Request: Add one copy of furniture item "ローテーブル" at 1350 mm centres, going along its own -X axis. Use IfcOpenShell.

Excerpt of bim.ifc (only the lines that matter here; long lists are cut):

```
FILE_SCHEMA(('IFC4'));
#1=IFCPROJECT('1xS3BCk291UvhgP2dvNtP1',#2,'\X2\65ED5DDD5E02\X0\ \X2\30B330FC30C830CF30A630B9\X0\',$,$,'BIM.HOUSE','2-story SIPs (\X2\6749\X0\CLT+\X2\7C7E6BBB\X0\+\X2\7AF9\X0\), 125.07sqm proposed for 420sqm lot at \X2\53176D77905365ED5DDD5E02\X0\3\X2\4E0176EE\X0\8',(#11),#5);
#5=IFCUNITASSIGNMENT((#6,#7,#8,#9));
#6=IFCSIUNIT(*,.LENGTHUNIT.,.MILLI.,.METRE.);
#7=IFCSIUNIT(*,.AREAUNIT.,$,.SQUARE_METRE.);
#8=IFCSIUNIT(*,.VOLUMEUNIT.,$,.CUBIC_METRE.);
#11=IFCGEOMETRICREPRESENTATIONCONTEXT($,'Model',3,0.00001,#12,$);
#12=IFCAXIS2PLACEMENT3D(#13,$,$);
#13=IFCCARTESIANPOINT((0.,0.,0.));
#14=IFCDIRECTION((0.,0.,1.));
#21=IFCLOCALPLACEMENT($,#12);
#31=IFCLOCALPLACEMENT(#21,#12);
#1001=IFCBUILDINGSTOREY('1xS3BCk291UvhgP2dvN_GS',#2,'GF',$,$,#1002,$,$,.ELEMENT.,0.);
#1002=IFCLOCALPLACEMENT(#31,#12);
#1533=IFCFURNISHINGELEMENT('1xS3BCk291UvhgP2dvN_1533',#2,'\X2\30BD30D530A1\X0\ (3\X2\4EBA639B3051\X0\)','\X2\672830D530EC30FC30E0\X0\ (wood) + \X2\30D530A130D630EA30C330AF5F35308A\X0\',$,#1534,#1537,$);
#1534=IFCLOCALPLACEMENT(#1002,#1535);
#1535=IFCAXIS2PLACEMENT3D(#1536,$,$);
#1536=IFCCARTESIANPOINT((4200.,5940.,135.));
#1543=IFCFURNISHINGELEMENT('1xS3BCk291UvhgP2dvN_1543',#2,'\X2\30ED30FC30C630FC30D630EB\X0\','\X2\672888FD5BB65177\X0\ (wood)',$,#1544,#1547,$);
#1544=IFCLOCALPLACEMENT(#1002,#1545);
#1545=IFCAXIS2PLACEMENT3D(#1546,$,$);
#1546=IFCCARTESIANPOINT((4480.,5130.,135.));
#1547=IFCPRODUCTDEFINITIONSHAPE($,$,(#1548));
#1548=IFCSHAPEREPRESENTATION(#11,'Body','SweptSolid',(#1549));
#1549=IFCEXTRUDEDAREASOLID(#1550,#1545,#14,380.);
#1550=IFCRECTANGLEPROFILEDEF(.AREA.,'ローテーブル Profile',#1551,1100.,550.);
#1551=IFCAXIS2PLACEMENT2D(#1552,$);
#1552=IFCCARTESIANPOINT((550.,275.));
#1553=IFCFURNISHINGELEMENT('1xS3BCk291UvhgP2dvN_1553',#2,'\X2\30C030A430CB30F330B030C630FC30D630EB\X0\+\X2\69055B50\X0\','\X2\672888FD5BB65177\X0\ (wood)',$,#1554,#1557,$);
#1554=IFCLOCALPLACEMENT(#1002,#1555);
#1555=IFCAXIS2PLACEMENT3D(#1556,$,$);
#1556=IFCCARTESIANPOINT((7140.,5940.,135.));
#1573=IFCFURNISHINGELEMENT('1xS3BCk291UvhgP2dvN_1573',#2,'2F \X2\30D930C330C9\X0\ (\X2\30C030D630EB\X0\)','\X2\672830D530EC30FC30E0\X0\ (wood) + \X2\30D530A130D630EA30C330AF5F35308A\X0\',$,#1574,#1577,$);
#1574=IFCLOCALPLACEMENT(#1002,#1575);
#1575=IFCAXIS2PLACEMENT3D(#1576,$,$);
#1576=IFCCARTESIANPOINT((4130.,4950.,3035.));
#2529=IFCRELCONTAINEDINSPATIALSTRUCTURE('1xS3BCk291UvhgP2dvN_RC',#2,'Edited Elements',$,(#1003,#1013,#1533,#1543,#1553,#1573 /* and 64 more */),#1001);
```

```python
import ifcopenshell
import ifcopenshell.api.geometry
import ifcopenshell.api.root
import ifcopenshell.util.element
import ifcopenshell.util.placement

model = ifcopenshell.open("bim.ifc")


def reuse_history(source, copy):
    """copy_class also copies each property set's owner history, people and application; keep the originals."""
    for rel in copy.IsDefinedBy:
        if rel.is_a("IfcRelDefinesByProperties") and (history := rel.RelatingPropertyDefinition.OwnerHistory):
            rel.RelatingPropertyDefinition.OwnerHistory = source.OwnerHistory
            ifcopenshell.util.element.remove_deep2(model, history)


source = model.by_guid("1xS3BCk291UvhgP2dvN_1543")
base = ifcopenshell.util.placement.get_local_placement(source.ObjectPlacement)
step = -base[:3, 0] * 1350.0

for i in range(1, 2):
    copy = ifcopenshell.api.root.copy_class(model, product=source)
    copy.Representation = ifcopenshell.util.element.copy_deep(
        model, source.Representation, exclude=["IfcGeometricRepresentationContext", "IfcRepresentationMap"]
    )
    reuse_history(source, copy)
    matrix = base.copy()
    matrix[:3, 3] += i * step
    print("added at", matrix[:3, 3].round(3) + 0.0)
    ifcopenshell.api.geometry.edit_object_placement(model, product=copy, matrix=matrix, is_si=False)

model.write("bim_edited.ifc")
```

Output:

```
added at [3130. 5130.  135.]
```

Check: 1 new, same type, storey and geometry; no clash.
